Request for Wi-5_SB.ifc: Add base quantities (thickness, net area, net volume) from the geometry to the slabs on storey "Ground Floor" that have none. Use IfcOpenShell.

First a look at what the model holds.

```python
import ifcopenshell
import ifcopenshell.util.element
import ifcopenshell.util.unit

model = ifcopenshell.open("Wi-5_SB.ifc")
print(model.schema)
for unit_type in ("LENGTHUNIT", "AREAUNIT", "VOLUMEUNIT"):
    print(unit_type, ifcopenshell.util.unit.calculate_unit_scale(model, unit_type))
storey = next(s for s in model.by_type("IfcBuildingStorey") if s.Name == "Ground Floor")
slabs = [e for e in ifcopenshell.util.element.get_decomposition(storey) if e.is_a("IfcSlab")]
for e in sorted(slabs, key=lambda e: e.id()):
    print(e.id(), e.is_a(), e.Name, list(ifcopenshell.util.element.get_psets(e, qtos_only=True)), sep=" | ")
```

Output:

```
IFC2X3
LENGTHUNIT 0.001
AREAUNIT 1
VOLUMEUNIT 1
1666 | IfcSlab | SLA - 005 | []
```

```python
import ifcopenshell
import ifcopenshell.api.pset
import ifcopenshell.geom
import ifcopenshell.util.element
import ifcopenshell.util.shape
import ifcopenshell.util.unit

model = ifcopenshell.open("Wi-5_SB.ifc")
unit_scale = ifcopenshell.util.unit.calculate_unit_scale(model)
area_scale = ifcopenshell.util.unit.calculate_unit_scale(model, "AREAUNIT")
volume_scale = ifcopenshell.util.unit.calculate_unit_scale(model, "VOLUMEUNIT")
settings = ifcopenshell.geom.settings()

storey = next(s for s in model.by_type("IfcBuildingStorey") if s.Name == "Ground Floor")
slabs = [e for e in ifcopenshell.util.element.get_decomposition(storey) if e.is_a("IfcSlab")]

for e in sorted(slabs, key=lambda e: e.id()):
    if ifcopenshell.util.element.get_psets(e, qtos_only=True, should_inherit=False):
        continue
    # Geometry comes back in metres, in the element's own axes.
    shape = ifcopenshell.geom.create_shape(settings, e)
    values = {
        "Width": ifcopenshell.util.shape.get_z(shape.geometry) / unit_scale,
        "NetArea": ifcopenshell.util.shape.get_footprint_area(shape.geometry) / area_scale,
        "NetVolume": ifcopenshell.util.shape.get_volume(shape.geometry) / volume_scale,
    }
    qto = ifcopenshell.api.pset.add_qto(model, product=e, name="BaseQuantities")
    ifcopenshell.api.pset.edit_qto(model, qto=qto, properties=values)
    print(e.id(), {k: round(v, 3) for k, v in values.items()})

model.write("Wi-5_SB_updated.ifc")
```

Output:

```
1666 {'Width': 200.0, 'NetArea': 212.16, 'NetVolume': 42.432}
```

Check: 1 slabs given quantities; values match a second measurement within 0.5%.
